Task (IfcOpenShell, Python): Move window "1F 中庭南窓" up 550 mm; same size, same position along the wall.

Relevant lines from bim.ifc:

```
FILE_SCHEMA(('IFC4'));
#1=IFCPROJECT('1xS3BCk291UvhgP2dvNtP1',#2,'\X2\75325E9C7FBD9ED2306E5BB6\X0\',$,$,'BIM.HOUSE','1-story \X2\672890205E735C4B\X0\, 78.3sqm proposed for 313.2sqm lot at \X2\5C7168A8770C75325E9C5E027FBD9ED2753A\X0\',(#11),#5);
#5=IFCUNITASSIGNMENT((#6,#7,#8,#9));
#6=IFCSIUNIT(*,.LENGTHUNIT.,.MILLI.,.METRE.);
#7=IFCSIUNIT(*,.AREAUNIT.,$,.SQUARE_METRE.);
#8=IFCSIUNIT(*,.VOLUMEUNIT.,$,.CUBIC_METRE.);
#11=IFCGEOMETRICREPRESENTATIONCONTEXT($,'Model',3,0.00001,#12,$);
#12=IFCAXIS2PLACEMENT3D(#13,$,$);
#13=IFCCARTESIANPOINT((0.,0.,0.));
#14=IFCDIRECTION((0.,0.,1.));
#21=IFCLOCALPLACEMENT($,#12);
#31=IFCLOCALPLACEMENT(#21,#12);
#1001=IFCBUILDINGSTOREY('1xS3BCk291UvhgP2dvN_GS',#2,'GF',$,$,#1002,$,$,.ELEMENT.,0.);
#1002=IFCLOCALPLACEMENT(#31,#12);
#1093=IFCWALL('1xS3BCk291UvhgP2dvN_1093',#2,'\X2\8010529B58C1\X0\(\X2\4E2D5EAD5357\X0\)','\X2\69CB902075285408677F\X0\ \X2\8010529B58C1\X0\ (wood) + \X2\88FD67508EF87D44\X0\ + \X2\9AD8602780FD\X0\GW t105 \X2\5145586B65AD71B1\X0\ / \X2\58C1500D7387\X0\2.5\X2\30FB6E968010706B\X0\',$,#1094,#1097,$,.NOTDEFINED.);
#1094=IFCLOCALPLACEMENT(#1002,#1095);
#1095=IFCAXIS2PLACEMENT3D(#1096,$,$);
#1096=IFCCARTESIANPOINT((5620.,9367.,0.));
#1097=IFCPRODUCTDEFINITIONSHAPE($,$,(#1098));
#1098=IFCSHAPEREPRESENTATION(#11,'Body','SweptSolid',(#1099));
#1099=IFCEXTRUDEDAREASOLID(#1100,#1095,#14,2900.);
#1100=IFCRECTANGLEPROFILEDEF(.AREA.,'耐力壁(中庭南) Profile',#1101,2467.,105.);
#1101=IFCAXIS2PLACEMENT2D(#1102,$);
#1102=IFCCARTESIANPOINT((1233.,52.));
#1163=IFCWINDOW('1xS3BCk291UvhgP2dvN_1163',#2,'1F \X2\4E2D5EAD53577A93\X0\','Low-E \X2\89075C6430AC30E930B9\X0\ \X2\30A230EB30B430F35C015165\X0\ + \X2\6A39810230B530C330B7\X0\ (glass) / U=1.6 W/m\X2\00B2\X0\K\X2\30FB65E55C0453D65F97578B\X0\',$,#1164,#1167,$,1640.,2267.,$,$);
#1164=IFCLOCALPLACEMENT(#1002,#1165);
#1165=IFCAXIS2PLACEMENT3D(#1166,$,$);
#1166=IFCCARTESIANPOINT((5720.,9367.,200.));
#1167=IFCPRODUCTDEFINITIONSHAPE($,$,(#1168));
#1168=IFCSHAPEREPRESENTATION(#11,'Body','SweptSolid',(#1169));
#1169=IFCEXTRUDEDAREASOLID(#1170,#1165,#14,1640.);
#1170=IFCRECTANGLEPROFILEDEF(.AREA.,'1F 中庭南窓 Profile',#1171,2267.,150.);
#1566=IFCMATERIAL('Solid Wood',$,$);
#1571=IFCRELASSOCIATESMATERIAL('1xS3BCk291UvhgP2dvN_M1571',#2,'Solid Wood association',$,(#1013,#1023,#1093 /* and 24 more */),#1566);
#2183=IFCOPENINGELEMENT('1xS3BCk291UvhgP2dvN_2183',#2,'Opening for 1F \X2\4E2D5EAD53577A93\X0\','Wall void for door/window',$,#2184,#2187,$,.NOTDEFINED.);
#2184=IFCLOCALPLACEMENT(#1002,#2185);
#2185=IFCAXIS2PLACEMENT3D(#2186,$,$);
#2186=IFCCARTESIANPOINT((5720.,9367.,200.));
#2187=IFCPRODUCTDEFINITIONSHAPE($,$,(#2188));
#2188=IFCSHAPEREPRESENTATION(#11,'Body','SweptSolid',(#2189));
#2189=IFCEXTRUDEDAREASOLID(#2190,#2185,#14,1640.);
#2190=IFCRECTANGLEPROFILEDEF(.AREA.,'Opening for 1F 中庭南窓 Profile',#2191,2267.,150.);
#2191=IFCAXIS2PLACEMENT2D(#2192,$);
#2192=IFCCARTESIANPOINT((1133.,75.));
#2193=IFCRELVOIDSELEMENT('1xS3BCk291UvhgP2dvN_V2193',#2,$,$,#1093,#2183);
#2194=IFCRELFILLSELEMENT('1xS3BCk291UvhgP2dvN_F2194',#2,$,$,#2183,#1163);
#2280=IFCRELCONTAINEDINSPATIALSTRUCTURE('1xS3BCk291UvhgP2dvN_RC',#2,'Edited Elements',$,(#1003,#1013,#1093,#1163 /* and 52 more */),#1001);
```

```python
import numpy as np
import ifcopenshell
import ifcopenshell.api.geometry
import ifcopenshell.util.placement
import ifcopenshell.util.unit

model = ifcopenshell.open("bim.ifc")
unit_scale = ifcopenshell.util.unit.calculate_unit_scale(model)

window = model.by_guid("1xS3BCk291UvhgP2dvN_1163")
opening = window.FillsVoids[0].RelatingOpeningElement
dz = 0.55 / unit_scale

shift = np.array([0.0, 0.0, dz])
# The window is not placed relative to its opening, so move both.
for product in (opening, window):
    matrix = ifcopenshell.util.placement.get_local_placement(product.ObjectPlacement)
    matrix[:3, 3] += shift
    ifcopenshell.api.geometry.edit_object_placement(model, product=product, matrix=matrix, is_si=False)

print(f"moved by {dz * unit_scale:+.3f} m")

model.write("bim-out.ifc")
```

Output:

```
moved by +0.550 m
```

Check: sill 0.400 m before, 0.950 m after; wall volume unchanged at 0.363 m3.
